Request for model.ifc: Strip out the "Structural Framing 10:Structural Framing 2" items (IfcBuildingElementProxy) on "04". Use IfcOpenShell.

First a look at what the model holds.

```python
import ifcopenshell
import ifcopenshell.util.element

model = ifcopenshell.open("model.ifc")
print(model.schema)
storey = next(s for s in model.by_type("IfcBuildingStorey") if s.Name == "04")
proxies = [e for e in ifcopenshell.util.element.get_decomposition(storey) if e.is_a("IfcBuildingElementProxy")]
seen = {}
for e in proxies:
    element_type = ifcopenshell.util.element.get_type(e)
    name = element_type.Name if element_type not in (None, e) else None
    seen[name] = seen.get(name, 0) + 1
for name, count in sorted(seen.items(), key=str):
    print(count, "x", name)
```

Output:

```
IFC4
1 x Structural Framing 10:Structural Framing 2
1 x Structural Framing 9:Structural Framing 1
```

```python
import ifcopenshell
import ifcopenshell.api.root
import ifcopenshell.util.element

model = ifcopenshell.open("model.ifc")

storey = next(s for s in model.by_type("IfcBuildingStorey") if s.Name == "04")
proxies = [e for e in ifcopenshell.util.element.get_decomposition(storey) if e.is_a("IfcBuildingElementProxy")]
targets = [e for e in proxies if (t := ifcopenshell.util.element.get_type(e)) not in (None, e) and t.Name == "Structural Framing 10:Structural Framing 2"]

for e in targets:
    ifcopenshell.api.root.remove_product(model, product=e)
print(len(targets), "removed")

model.write("model_edited.ifc")
```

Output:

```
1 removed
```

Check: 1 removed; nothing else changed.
